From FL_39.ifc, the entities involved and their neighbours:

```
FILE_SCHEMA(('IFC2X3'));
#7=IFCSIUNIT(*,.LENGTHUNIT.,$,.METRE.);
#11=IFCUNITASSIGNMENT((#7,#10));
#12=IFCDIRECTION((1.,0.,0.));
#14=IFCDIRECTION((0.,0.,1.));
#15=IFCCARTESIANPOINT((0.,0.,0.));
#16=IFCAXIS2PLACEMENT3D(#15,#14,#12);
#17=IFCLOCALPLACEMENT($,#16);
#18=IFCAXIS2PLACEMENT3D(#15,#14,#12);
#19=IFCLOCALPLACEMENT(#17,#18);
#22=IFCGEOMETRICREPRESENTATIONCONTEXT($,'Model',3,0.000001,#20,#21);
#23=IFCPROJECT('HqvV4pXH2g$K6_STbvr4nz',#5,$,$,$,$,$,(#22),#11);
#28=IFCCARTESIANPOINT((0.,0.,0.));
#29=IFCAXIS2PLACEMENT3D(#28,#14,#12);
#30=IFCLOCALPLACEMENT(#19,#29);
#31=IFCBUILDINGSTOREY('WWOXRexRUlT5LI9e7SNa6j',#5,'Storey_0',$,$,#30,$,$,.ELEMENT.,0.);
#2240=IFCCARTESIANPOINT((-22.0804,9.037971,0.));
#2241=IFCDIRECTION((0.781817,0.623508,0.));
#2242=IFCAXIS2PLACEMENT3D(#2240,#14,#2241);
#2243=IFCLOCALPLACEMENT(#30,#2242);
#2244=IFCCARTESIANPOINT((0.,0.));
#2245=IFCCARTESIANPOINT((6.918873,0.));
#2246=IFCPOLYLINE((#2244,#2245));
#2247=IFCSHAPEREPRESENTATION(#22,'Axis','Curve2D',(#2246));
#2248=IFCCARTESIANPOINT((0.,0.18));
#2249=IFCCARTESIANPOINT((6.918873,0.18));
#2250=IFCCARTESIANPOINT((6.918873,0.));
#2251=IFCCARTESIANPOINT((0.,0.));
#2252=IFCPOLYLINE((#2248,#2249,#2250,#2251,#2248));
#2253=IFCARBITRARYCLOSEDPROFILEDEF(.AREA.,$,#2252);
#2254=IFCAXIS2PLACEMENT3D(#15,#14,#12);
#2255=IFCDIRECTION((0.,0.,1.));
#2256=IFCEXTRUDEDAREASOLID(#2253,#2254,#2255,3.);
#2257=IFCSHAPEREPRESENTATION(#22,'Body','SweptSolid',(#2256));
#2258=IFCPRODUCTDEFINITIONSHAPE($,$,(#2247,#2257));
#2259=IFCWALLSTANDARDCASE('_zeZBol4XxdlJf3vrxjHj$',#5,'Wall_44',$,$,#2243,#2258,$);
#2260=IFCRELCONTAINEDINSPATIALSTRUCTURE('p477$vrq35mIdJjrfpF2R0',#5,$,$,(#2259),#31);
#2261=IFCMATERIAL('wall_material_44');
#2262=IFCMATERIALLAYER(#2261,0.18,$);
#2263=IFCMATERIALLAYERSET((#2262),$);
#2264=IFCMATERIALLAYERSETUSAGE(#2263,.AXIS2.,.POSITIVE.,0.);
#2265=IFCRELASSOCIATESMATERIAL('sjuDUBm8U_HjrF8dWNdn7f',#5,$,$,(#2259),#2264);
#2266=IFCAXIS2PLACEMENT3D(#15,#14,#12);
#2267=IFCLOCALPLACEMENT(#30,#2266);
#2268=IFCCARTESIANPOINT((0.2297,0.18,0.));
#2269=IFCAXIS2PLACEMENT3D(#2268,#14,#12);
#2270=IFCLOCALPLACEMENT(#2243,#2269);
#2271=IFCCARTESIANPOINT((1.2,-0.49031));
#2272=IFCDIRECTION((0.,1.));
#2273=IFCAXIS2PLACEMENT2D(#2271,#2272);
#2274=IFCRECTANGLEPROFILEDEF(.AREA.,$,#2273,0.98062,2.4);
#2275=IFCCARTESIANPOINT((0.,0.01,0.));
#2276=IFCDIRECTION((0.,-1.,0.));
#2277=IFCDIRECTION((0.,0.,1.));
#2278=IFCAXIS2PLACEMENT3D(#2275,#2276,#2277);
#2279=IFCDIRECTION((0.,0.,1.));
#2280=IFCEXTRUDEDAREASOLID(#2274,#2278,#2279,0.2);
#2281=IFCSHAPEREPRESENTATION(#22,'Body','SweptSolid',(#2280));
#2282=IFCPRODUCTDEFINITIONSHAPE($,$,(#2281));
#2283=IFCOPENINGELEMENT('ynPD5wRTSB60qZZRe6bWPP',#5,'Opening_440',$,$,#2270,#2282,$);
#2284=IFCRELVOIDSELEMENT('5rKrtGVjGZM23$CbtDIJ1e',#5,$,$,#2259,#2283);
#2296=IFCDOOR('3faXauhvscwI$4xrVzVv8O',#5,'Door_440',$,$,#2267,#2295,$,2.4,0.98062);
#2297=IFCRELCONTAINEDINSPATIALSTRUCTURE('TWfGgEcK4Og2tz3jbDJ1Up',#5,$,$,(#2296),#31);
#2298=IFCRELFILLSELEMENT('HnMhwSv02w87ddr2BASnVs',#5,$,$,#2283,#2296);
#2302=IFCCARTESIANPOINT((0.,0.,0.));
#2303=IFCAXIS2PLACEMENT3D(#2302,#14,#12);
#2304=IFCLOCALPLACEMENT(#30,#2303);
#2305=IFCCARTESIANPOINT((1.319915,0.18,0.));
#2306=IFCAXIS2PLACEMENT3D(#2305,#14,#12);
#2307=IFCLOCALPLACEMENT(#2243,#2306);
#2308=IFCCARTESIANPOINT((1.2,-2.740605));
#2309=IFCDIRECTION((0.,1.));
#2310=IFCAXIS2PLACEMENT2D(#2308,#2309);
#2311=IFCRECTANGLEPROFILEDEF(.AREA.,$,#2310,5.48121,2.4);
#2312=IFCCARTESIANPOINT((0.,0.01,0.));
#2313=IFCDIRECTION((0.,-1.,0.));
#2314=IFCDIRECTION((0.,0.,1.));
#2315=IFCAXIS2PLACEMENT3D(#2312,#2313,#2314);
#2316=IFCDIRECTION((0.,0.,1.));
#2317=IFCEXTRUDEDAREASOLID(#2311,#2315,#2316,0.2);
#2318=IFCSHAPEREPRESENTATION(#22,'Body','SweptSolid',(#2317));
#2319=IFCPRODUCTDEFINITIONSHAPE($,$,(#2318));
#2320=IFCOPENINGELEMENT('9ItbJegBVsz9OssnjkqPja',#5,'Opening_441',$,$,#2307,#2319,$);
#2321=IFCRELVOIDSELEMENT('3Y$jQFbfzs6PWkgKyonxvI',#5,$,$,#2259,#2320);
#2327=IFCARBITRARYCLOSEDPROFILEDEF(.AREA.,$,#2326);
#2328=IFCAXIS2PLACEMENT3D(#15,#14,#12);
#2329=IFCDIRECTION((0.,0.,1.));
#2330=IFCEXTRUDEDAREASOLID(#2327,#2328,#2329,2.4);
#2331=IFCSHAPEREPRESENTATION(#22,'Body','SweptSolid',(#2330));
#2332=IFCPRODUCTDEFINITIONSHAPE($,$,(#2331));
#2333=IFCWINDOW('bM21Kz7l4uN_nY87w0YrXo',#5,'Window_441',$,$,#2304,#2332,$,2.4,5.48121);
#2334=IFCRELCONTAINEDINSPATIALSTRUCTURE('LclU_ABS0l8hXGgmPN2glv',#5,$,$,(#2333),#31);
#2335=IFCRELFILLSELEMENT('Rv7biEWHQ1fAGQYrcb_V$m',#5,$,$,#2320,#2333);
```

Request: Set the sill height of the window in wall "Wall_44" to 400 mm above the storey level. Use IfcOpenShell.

```python
import numpy as np
import ifcopenshell
import ifcopenshell.api.geometry
import ifcopenshell.geom
import ifcopenshell.util.element
import ifcopenshell.util.placement
import ifcopenshell.util.shape
import ifcopenshell.util.unit

model = ifcopenshell.open("FL_39.ifc")
unit_scale = ifcopenshell.util.unit.calculate_unit_scale(model)

window = model.by_id(2333)
opening = window.FillsVoids[0].RelatingOpeningElement
storey = ifcopenshell.util.element.get_container(window, ifc_class="IfcBuildingStorey")
level = ifcopenshell.util.placement.get_local_placement(storey.ObjectPlacement)[2, 3]

# The opening's origin need not be at the sill, so measure its lowest point.
shape = ifcopenshell.geom.create_shape(ifcopenshell.geom.settings(), opening)
bottom = ifcopenshell.util.shape.get_shape_bottom_elevation(shape, shape.geometry) / unit_scale
dz = level + 0.4 / unit_scale - bottom

shift = np.array([0.0, 0.0, dz])
# The window is not placed relative to its opening, so move both.
for product in (opening, window):
    matrix = ifcopenshell.util.placement.get_local_placement(product.ObjectPlacement)
    matrix[:3, 3] += shift
    ifcopenshell.api.geometry.edit_object_placement(model, product=product, matrix=matrix, is_si=False)

print(f"moved by {dz * unit_scale:+.3f} m")

model.write("FL_39_v2.ifc")
```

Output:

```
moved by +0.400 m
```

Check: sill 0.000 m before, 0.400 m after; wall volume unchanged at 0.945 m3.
